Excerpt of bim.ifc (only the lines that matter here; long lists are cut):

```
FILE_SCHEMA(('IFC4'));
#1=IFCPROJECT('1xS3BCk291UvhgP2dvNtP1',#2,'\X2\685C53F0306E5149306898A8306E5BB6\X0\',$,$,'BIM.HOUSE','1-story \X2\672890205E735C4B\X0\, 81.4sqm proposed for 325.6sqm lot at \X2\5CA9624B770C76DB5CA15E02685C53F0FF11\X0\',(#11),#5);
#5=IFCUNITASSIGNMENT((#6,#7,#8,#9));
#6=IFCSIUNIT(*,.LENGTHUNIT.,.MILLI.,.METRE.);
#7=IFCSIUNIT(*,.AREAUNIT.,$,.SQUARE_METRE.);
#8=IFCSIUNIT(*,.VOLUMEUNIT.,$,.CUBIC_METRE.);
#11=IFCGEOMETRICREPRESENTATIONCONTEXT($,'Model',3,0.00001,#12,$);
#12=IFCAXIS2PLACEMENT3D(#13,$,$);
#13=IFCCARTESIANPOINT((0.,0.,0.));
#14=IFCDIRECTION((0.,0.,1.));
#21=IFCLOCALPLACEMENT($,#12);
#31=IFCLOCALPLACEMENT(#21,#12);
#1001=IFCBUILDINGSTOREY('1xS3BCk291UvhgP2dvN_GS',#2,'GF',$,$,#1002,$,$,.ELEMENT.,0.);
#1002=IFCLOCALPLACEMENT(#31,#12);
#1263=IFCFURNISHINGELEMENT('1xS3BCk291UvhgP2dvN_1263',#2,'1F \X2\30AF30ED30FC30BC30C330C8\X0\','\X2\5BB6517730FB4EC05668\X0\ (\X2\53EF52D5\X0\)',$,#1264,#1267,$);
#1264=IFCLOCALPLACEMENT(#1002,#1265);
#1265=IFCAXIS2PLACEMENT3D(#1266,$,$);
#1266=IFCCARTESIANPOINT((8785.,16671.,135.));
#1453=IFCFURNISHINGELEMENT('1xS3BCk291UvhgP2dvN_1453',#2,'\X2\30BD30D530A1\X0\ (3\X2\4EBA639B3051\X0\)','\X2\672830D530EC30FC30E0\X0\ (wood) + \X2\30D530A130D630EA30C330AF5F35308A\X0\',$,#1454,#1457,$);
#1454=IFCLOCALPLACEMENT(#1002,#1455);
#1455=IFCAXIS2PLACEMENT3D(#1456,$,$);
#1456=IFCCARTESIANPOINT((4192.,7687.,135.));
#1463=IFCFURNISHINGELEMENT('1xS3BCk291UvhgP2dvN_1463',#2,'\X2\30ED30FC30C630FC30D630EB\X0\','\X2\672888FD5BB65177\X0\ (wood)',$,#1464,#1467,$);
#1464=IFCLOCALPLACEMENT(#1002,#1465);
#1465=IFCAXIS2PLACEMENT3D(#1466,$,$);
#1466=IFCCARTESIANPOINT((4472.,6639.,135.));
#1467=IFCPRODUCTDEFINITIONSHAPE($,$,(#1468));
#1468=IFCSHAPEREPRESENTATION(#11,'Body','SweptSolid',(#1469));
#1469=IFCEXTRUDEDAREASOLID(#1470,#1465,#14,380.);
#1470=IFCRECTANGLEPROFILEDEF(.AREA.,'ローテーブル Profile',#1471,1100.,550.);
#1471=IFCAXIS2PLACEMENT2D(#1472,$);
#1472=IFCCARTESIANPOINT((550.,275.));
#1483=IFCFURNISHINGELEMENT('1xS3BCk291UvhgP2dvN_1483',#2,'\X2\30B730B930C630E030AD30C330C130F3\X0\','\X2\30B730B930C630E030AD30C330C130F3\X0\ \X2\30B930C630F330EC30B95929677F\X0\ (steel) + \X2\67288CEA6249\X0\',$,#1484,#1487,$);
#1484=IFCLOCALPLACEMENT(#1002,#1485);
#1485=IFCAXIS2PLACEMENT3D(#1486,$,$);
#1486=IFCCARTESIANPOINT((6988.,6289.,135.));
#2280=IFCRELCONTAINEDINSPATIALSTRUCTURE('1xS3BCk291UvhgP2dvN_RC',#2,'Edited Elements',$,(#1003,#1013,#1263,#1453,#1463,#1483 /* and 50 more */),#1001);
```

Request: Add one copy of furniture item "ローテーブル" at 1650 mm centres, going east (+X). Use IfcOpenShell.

```python
import numpy as np
import ifcopenshell
import ifcopenshell.api.geometry
import ifcopenshell.api.root
import ifcopenshell.util.element
import ifcopenshell.util.placement
import ifcopenshell.util.unit

model = ifcopenshell.open("bim.ifc")
unit_scale = ifcopenshell.util.unit.calculate_unit_scale(model)


def reuse_history(source, copy):
    """copy_class also copies each property set's owner history, people and application; keep the originals."""
    for rel in copy.IsDefinedBy:
        if rel.is_a("IfcRelDefinesByProperties") and (history := rel.RelatingPropertyDefinition.OwnerHistory):
            rel.RelatingPropertyDefinition.OwnerHistory = source.OwnerHistory
            ifcopenshell.util.element.remove_deep2(model, history)


source = model.by_id(1463)
base = ifcopenshell.util.placement.get_local_placement(source.ObjectPlacement)
step = np.array([1.0, 0.0, 0.0]) * 1.65 / unit_scale

for i in range(1, 2):
    copy = ifcopenshell.api.root.copy_class(model, product=source)
    copy.Representation = ifcopenshell.util.element.copy_deep(
        model, source.Representation, exclude=["IfcGeometricRepresentationContext", "IfcRepresentationMap"]
    )
    reuse_history(source, copy)
    matrix = base.copy()
    matrix[:3, 3] += i * step
    print("added at", matrix[:3, 3].round(3) + 0.0)
    ifcopenshell.api.geometry.edit_object_placement(model, product=copy, matrix=matrix, is_si=False)

model.write("bim_v2.ifc")
```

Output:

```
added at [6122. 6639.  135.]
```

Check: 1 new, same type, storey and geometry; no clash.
